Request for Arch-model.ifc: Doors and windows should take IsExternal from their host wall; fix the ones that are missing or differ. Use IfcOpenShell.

First a look at what the model holds.

```python
import ifcopenshell
import ifcopenshell.util.element

model = ifcopenshell.open("Arch-model.ifc")
print(model.schema)
seen = {}
for e in model.by_type("IfcDoor") + model.by_type("IfcWindow"):
    if not e.FillsVoids:
        continue
    host = e.FillsVoids[0].RelatingOpeningElement.VoidsElements[0].RelatingBuildingElement
    own = ifcopenshell.util.element.get_pset(e, f"Pset_{e.is_a()[3:].removesuffix('StandardCase')}Common", "IsExternal")
    wall = ifcopenshell.util.element.get_pset(host, "Pset_WallCommon", "IsExternal")
    seen[e.is_a(), own, wall] = seen.get((e.is_a(), own, wall), 0) + 1
for (cls, own, wall), count in sorted(seen.items(), key=str):
    print(count, cls, "IsExternal:", own, "| host wall:", wall)
```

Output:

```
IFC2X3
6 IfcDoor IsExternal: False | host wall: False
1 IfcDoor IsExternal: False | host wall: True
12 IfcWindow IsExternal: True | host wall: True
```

```python
import ifcopenshell
import ifcopenshell.api.pset
import ifcopenshell.util.element

model = ifcopenshell.open("Arch-model.ifc")

count = 0
for ifc_class, pset_name in (("IfcDoor", "Pset_DoorCommon"), ("IfcWindow", "Pset_WindowCommon")):
    for e in model.by_type(ifc_class):
        if not e.FillsVoids:
            continue
        host = e.FillsVoids[0].RelatingOpeningElement.VoidsElements[0].RelatingBuildingElement
        external = ifcopenshell.util.element.get_pset(host, "Pset_WallCommon", "IsExternal")
        if external is None or ifcopenshell.util.element.get_pset(e, pset_name, "IsExternal") == external:
            continue
        pset = ifcopenshell.api.pset.add_pset(model, product=e, name=pset_name)
        ifcopenshell.api.pset.edit_pset(model, pset=pset, properties={"IsExternal": external})
        count += 1

print(count, "updated")

model.write("Arch-model-out.ifc")
```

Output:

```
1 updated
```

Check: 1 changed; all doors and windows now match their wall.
